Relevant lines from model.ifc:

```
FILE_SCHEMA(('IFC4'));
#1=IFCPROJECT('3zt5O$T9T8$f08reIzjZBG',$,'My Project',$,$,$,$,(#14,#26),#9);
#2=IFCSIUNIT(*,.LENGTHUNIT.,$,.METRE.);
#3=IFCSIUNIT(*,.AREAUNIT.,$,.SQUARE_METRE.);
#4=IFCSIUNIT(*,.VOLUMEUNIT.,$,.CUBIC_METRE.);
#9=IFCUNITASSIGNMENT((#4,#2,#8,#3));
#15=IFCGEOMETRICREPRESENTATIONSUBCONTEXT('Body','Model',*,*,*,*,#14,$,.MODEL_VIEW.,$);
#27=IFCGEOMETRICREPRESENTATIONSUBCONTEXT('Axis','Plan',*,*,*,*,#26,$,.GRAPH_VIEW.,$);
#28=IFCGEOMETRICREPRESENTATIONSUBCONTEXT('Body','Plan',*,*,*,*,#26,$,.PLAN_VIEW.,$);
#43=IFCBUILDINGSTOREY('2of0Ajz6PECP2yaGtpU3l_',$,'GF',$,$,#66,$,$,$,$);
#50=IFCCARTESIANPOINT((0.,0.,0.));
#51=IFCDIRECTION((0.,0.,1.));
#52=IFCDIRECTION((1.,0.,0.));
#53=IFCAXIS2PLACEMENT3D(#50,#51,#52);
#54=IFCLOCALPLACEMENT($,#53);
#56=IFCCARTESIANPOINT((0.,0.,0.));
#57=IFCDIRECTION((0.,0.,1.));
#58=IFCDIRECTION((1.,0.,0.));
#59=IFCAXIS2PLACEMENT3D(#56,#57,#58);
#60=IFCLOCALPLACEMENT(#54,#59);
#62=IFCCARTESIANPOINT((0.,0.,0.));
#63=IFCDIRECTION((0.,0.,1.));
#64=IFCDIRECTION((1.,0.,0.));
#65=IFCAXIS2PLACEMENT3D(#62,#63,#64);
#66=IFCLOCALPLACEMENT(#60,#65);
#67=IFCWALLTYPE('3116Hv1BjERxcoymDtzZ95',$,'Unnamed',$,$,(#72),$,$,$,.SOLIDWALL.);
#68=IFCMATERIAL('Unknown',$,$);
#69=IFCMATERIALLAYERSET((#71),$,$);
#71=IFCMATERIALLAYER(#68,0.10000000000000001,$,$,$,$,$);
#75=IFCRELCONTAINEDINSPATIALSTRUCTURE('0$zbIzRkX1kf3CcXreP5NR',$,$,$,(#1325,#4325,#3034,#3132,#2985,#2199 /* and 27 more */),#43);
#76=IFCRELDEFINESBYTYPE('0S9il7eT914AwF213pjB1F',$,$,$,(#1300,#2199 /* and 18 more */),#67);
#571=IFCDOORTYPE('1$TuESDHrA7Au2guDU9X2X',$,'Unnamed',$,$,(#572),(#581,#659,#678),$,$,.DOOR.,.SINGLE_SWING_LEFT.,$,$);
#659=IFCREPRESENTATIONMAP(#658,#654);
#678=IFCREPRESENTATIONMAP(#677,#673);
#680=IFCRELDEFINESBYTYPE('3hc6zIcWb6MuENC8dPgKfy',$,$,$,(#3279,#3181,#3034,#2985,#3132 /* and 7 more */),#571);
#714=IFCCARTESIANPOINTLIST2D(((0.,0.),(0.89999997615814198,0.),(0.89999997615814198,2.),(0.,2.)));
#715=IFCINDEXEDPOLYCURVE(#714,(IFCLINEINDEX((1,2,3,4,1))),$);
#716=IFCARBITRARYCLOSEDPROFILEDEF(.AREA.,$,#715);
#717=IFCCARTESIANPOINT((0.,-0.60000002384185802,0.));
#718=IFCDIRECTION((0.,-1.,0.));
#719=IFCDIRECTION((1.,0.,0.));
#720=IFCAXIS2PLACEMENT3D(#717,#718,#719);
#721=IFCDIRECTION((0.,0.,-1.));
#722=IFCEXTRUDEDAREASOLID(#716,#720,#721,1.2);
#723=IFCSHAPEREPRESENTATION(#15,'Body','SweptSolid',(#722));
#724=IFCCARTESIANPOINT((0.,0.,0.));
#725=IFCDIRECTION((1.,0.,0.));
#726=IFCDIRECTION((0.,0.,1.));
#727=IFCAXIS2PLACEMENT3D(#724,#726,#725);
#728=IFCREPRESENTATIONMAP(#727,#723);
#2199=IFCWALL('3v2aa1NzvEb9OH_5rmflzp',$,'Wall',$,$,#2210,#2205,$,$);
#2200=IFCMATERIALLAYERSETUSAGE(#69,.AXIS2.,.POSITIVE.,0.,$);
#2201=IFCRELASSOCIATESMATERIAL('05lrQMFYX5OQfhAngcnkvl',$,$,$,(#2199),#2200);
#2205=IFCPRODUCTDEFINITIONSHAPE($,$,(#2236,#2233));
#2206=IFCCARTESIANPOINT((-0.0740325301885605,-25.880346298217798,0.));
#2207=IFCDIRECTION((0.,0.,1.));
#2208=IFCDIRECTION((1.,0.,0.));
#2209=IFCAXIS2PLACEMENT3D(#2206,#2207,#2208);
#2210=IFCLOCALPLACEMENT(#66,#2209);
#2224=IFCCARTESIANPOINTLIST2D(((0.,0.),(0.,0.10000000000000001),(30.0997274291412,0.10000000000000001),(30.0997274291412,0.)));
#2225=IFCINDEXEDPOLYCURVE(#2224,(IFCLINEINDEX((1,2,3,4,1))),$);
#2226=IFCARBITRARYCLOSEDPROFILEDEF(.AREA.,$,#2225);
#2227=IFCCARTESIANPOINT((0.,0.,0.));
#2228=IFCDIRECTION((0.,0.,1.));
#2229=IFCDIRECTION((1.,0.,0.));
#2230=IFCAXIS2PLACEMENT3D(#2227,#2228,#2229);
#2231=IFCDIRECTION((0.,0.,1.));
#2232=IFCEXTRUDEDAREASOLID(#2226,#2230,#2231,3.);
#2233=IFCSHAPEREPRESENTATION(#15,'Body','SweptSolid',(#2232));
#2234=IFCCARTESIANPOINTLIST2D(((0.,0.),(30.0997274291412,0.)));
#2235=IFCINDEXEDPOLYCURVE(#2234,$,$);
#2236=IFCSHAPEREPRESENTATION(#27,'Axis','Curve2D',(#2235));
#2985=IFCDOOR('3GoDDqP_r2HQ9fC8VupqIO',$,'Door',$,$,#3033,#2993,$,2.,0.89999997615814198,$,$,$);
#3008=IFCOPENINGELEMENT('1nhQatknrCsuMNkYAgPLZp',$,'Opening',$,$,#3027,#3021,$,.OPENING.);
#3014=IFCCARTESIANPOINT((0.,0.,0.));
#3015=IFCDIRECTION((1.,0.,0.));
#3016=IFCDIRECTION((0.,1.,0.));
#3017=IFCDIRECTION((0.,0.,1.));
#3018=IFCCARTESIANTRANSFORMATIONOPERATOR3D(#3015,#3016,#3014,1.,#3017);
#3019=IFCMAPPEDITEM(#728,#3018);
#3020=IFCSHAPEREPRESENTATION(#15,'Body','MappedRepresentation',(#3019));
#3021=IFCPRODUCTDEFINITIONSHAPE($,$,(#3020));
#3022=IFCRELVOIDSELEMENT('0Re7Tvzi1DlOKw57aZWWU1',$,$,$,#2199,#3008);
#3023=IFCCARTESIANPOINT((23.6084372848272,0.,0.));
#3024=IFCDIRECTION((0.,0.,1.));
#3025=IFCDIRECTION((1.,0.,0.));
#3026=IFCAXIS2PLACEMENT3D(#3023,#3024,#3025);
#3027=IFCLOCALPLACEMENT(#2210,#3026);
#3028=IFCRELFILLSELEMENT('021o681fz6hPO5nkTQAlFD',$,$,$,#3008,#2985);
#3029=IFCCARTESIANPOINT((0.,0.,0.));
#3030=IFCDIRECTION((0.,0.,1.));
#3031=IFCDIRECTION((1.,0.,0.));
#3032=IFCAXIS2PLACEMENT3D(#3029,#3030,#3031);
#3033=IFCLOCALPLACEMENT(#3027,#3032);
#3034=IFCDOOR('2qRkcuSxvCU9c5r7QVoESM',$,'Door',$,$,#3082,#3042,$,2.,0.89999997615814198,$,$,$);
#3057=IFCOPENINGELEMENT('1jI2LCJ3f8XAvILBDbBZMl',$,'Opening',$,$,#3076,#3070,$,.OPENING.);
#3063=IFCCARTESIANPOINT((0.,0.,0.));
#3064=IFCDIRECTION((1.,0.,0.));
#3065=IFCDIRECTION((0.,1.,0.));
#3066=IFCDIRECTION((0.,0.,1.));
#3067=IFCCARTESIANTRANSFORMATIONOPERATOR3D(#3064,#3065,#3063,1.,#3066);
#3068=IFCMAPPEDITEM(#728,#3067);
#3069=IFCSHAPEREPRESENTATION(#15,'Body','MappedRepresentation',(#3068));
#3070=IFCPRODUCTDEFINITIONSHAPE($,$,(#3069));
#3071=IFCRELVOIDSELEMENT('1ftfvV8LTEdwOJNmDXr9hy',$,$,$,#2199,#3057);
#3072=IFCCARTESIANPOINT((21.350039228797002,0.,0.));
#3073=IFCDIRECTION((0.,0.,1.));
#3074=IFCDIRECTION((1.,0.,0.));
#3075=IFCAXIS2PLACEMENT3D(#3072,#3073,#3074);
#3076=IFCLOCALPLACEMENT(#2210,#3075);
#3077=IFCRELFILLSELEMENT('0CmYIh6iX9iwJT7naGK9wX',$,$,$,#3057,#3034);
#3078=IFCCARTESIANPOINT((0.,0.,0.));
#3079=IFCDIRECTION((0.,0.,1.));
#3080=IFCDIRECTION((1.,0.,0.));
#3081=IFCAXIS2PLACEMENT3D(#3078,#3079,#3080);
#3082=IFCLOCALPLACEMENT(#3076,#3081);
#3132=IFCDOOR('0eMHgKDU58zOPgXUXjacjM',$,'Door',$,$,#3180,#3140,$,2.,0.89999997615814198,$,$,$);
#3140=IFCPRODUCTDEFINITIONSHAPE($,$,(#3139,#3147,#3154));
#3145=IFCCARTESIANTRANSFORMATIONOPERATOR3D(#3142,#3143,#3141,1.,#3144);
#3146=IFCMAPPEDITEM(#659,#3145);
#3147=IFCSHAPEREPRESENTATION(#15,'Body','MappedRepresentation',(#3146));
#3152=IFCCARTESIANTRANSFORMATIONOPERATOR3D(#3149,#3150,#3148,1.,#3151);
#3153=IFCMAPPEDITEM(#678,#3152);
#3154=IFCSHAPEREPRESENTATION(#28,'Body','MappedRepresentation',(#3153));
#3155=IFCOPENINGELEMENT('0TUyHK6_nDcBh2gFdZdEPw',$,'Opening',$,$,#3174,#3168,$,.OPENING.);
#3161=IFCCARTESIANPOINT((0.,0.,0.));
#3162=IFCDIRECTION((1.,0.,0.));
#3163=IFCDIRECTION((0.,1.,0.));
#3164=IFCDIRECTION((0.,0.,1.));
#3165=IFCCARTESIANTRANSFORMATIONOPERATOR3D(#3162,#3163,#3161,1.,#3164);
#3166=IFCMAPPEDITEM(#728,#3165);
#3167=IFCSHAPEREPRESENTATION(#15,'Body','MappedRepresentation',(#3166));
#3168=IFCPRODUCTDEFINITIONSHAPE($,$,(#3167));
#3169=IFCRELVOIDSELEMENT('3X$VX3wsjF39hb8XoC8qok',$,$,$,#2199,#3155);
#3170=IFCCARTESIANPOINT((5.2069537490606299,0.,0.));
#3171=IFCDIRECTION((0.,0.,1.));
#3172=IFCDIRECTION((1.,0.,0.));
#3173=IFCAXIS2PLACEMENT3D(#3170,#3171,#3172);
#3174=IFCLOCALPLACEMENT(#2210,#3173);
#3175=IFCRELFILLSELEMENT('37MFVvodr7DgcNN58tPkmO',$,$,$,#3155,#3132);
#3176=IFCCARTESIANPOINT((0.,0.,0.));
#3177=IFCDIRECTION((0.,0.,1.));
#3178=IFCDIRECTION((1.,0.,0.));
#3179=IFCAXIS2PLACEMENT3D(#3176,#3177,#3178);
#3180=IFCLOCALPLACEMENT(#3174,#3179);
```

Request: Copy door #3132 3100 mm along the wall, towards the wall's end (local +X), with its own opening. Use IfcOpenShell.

```python
import ifcopenshell
import ifcopenshell.api.feature
import ifcopenshell.api.geometry
import ifcopenshell.api.root
import ifcopenshell.geom
import ifcopenshell.util.element
import ifcopenshell.util.placement
import ifcopenshell.util.shape
import ifcopenshell.util.unit

model = ifcopenshell.open("model.ifc")
unit_scale = ifcopenshell.util.unit.calculate_unit_scale(model)
settings = ifcopenshell.geom.settings()


def volume(element):
    """Net volume in cubic metres, openings subtracted."""
    shape = ifcopenshell.geom.create_shape(settings, element)
    return ifcopenshell.util.shape.get_volume(shape.geometry)


door = model.by_guid("0eMHgKDU58zOPgXUXjacjM")
opening = door.FillsVoids[0].RelatingOpeningElement
wall = opening.VoidsElements[0].RelatingBuildingElement
before = volume(wall)
shift = ifcopenshell.util.placement.get_local_placement(wall.ObjectPlacement)[:3, 0] * 3.1 / unit_scale

# copy_class copies the void relationship, type, container and properties, but no geometry.
new_opening = ifcopenshell.api.root.copy_class(model, product=opening)
new_opening.Representation = ifcopenshell.util.element.copy_deep(
    model, opening.Representation, exclude=["IfcGeometricRepresentationContext", "IfcRepresentationMap"]
)
new_door = ifcopenshell.api.root.copy_class(model, product=door)
new_door.Representation = ifcopenshell.util.element.copy_deep(
    model, door.Representation, exclude=["IfcGeometricRepresentationContext", "IfcRepresentationMap"]
)
ifcopenshell.api.feature.add_filling(model, opening=new_opening, element=new_door)

for old, new in ((opening, new_opening), (door, new_door)):
    matrix = ifcopenshell.util.placement.get_local_placement(old.ObjectPlacement)
    matrix[:3, 3] += shift
    ifcopenshell.api.geometry.edit_object_placement(model, product=new, matrix=matrix, is_si=False)

after = volume(wall)

print(f"wall volume {before:.3f} -> {after:.3f} m3")

model.write("model_updated.ifc")
```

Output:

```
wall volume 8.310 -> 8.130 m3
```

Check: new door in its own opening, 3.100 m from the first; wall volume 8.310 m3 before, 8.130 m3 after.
